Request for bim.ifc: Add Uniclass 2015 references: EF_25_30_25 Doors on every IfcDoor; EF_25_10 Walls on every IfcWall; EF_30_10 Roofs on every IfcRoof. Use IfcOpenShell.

First a look at what the model holds.

```python
import ifcopenshell

model = ifcopenshell.open("bim.ifc")
print(model.schema)
print("classifications:", [c.Name for c in model.by_type("IfcClassification")])
for ifc_class in ("IfcDoor", "IfcRoof", "IfcStair", "IfcWall", "IfcWindow"):
    print(ifc_class, len(model.by_type(ifc_class)))
```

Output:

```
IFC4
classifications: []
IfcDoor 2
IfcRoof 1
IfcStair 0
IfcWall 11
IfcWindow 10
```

```python
import ifcopenshell
import ifcopenshell.api.classification

model = ifcopenshell.open("bim.ifc")

system = ifcopenshell.api.classification.add_classification(model, classification="Uniclass 2015")

codes = {
    "IfcDoor": ("EF_25_30_25", "Doors"),
    "IfcWall": ("EF_25_10", "Walls"),
    "IfcRoof": ("EF_30_10", "Roofs"),
}
for ifc_class, (code, name) in codes.items():
    products = model.by_type(ifc_class)
    ifcopenshell.api.classification.add_reference(
        model, products=products, classification=system, identification=code, name=name
    )
    print(code, len(products))

model.write("bim_v2.ifc")
```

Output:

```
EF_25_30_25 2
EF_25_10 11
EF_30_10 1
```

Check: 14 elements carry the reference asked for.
